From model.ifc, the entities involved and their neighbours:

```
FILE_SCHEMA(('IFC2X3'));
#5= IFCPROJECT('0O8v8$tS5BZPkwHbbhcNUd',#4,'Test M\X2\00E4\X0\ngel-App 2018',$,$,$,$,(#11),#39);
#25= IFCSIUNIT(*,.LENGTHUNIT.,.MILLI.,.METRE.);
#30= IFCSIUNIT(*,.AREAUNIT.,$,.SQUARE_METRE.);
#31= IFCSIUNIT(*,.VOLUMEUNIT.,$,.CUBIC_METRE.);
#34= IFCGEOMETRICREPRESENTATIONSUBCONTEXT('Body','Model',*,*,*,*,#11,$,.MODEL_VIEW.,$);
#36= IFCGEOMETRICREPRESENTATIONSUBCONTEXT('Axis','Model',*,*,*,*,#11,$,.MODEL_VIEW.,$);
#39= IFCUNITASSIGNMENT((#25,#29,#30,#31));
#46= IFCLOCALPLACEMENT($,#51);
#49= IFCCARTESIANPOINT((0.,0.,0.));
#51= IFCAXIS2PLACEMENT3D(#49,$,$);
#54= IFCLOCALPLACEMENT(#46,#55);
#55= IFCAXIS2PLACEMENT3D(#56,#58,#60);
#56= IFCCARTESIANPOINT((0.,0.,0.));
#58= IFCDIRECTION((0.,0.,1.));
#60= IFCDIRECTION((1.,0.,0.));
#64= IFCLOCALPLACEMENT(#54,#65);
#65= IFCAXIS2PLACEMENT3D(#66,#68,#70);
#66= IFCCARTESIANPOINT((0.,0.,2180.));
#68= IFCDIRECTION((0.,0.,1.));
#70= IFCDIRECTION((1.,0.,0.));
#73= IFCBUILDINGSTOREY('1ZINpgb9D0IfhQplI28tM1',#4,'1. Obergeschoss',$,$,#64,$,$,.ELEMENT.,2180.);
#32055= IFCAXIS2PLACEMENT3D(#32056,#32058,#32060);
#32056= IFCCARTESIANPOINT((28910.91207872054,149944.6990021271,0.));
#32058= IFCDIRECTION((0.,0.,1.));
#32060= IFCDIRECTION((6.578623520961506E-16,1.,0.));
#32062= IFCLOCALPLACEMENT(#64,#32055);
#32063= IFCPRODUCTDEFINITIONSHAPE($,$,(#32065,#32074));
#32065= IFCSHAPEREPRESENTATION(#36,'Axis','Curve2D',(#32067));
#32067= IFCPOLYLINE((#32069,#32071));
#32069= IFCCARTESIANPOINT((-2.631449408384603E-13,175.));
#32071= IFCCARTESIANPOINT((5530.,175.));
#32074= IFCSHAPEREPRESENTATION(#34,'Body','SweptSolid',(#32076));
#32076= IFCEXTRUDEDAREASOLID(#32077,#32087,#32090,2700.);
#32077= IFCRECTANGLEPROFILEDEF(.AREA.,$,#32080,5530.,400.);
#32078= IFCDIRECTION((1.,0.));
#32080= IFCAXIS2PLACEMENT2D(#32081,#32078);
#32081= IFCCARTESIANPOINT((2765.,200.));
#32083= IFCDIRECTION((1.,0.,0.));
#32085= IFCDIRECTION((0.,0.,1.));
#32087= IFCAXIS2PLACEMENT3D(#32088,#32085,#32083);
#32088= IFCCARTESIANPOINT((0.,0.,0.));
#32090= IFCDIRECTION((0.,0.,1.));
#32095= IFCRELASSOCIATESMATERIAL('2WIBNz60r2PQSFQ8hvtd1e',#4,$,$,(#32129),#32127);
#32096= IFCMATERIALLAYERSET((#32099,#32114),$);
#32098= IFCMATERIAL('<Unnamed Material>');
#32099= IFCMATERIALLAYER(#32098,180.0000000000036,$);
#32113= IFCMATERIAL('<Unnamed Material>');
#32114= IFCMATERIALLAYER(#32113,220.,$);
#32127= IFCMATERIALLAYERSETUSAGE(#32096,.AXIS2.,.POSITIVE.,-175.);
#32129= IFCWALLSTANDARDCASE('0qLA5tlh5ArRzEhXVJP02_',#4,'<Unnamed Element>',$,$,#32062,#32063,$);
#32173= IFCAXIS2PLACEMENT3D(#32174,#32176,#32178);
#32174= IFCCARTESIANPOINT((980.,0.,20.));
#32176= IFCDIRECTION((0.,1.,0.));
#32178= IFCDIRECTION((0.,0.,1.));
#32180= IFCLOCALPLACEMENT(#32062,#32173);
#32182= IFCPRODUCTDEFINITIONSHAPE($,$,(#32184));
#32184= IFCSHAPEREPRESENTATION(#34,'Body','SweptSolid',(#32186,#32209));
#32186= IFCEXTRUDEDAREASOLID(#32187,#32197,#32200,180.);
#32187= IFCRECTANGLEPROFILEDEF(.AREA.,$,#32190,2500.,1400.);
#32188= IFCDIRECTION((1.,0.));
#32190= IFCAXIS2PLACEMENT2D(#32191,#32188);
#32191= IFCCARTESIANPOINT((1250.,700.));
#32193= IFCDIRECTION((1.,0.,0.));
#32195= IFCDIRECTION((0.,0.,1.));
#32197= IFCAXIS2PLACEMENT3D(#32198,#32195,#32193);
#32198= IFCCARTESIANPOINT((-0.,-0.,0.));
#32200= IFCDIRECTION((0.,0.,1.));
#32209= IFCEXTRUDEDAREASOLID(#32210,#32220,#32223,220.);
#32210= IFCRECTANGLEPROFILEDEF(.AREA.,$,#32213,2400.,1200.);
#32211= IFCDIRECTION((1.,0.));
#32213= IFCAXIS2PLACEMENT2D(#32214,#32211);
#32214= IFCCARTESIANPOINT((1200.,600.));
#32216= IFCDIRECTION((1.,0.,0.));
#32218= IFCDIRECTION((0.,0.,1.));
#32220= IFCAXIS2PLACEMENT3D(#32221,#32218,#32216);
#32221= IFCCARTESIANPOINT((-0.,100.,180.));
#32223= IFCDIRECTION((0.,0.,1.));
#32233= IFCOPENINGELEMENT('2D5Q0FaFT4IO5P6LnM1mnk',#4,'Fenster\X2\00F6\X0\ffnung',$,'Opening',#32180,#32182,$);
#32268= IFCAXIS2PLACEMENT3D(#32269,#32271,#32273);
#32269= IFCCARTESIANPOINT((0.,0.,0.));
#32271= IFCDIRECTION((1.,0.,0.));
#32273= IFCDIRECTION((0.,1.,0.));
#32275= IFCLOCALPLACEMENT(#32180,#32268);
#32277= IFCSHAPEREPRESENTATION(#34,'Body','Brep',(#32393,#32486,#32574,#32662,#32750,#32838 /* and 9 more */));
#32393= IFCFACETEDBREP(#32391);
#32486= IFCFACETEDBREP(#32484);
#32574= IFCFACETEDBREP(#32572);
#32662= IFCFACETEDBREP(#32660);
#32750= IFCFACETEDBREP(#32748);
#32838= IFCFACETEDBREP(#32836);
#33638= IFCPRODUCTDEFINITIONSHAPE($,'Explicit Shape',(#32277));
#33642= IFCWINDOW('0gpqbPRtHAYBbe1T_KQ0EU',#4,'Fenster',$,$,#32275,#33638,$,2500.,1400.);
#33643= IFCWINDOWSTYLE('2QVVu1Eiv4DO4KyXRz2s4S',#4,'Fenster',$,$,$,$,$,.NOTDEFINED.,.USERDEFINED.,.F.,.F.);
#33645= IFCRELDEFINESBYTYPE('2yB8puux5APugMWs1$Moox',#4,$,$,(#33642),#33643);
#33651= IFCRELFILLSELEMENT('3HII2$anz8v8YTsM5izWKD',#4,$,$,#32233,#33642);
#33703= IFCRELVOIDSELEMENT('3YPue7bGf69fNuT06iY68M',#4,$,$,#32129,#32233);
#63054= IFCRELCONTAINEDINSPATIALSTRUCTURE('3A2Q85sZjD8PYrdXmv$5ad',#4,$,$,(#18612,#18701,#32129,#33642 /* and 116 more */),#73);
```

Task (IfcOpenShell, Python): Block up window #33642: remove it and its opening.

```python
import ifcopenshell
import ifcopenshell.api.feature
import ifcopenshell.api.root
import ifcopenshell.geom
import ifcopenshell.util.shape

model = ifcopenshell.open("model.ifc")
settings = ifcopenshell.geom.settings()


def volume(element):
    """Net volume in cubic metres, openings subtracted."""
    shape = ifcopenshell.geom.create_shape(settings, element)
    return ifcopenshell.util.shape.get_volume(shape.geometry)


window = model.by_guid("0gpqbPRtHAYBbe1T_KQ0EU")
opening = window.FillsVoids[0].RelatingOpeningElement
wall = opening.VoidsElements[0].RelatingBuildingElement
before = volume(wall)

ifcopenshell.api.root.remove_product(model, product=window)
ifcopenshell.api.feature.remove_feature(model, feature=opening)

after = volume(wall)

print(f"wall volume {before:.3f} -> {after:.3f} m3")

model.write("model_rev.ifc")
```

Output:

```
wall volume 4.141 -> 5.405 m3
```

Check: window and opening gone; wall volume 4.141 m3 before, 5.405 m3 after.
